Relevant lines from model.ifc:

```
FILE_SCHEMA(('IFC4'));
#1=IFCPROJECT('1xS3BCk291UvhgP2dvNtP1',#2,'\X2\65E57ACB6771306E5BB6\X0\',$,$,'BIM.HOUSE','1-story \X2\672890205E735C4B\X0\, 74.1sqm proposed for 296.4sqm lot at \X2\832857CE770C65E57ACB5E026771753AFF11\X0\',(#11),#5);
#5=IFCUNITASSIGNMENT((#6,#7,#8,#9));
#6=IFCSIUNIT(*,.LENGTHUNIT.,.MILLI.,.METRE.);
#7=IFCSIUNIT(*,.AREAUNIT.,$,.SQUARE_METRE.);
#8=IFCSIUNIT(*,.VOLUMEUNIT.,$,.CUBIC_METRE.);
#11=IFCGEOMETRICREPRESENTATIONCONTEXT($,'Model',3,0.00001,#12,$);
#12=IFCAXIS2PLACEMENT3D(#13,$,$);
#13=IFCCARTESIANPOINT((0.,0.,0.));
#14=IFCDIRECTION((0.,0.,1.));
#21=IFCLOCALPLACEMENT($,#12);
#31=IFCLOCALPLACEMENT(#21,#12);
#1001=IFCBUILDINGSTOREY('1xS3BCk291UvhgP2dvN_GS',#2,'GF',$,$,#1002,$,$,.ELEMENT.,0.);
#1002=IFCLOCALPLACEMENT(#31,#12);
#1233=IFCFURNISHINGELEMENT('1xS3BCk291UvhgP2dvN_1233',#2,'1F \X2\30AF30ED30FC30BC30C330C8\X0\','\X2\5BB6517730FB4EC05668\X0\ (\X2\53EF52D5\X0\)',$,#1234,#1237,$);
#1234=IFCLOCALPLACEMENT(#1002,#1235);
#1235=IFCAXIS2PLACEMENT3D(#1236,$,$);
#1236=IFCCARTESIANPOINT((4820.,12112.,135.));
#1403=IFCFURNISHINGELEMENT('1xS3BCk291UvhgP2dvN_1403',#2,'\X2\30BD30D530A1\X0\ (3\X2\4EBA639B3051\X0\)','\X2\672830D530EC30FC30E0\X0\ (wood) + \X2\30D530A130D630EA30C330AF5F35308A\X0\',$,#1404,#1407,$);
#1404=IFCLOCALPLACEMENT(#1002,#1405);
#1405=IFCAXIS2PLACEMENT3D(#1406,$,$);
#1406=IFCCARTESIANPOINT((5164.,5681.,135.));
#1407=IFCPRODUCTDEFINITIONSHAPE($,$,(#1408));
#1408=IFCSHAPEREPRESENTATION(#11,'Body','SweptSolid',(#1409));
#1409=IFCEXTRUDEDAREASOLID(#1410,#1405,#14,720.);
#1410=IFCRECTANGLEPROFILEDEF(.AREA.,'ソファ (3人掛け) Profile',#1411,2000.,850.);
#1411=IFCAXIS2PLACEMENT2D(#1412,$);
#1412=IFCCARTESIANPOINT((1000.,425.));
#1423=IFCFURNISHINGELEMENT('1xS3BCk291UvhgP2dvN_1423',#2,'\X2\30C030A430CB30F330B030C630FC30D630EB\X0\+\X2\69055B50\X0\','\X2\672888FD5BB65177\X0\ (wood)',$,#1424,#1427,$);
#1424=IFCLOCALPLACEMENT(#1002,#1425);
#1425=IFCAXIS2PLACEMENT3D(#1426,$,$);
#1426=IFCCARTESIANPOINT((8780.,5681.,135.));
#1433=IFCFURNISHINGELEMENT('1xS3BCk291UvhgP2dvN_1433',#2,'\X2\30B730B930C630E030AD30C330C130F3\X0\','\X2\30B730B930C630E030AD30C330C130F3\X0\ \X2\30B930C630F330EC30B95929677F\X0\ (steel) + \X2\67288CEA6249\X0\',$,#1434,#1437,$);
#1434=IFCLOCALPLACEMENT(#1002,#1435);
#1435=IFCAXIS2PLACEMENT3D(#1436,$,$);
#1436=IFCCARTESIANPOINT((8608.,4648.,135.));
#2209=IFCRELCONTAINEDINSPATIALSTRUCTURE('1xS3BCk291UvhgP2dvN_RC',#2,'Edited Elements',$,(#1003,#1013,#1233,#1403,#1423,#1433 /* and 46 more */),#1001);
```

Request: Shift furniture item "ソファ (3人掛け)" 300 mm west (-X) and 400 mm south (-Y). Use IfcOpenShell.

```python
import ifcopenshell
import ifcopenshell.api.geometry
import ifcopenshell.util.placement

model = ifcopenshell.open("model.ifc")

item = model.by_guid("1xS3BCk291UvhgP2dvN_1403")
matrix = ifcopenshell.util.placement.get_local_placement(item.ObjectPlacement)
matrix[0, 3] -= 300.0
matrix[1, 3] -= 400.0
ifcopenshell.api.geometry.edit_object_placement(model, product=item, matrix=matrix, is_si=False)

print(ifcopenshell.util.placement.get_local_placement(item.ObjectPlacement).round(3) + 0.0)

model.write("model_v2.ifc")
```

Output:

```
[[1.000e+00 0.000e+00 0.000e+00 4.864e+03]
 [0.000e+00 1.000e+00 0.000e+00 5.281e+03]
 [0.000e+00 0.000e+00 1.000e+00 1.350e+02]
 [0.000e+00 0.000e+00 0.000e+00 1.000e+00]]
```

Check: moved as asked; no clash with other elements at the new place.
